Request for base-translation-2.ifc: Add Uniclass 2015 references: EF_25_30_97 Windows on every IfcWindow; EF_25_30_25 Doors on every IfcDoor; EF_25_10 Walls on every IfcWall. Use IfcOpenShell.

First a look at what the model holds.

```python
import ifcopenshell

model = ifcopenshell.open("base-translation-2.ifc")
print(model.schema)
print("classifications:", [c.Name for c in model.by_type("IfcClassification")])
for ifc_class in ("IfcDoor", "IfcRoof", "IfcStair", "IfcWall", "IfcWindow"):
    print(ifc_class, len(model.by_type(ifc_class)))
```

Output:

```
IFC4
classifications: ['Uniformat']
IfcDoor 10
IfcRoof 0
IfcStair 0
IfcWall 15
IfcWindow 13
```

```python
import ifcopenshell
import ifcopenshell.api.classification

model = ifcopenshell.open("base-translation-2.ifc")

system = ifcopenshell.api.classification.add_classification(model, classification="Uniclass 2015")

codes = {
    "IfcWindow": ("EF_25_30_97", "Windows"),
    "IfcDoor": ("EF_25_30_25", "Doors"),
    "IfcWall": ("EF_25_10", "Walls"),
}
for ifc_class, (code, name) in codes.items():
    products = model.by_type(ifc_class)
    ifcopenshell.api.classification.add_reference(
        model, products=products, classification=system, identification=code, name=name
    )
    print(code, len(products))

model.write("base-translation-2_updated.ifc")
```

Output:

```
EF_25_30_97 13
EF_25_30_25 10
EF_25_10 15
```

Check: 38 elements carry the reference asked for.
